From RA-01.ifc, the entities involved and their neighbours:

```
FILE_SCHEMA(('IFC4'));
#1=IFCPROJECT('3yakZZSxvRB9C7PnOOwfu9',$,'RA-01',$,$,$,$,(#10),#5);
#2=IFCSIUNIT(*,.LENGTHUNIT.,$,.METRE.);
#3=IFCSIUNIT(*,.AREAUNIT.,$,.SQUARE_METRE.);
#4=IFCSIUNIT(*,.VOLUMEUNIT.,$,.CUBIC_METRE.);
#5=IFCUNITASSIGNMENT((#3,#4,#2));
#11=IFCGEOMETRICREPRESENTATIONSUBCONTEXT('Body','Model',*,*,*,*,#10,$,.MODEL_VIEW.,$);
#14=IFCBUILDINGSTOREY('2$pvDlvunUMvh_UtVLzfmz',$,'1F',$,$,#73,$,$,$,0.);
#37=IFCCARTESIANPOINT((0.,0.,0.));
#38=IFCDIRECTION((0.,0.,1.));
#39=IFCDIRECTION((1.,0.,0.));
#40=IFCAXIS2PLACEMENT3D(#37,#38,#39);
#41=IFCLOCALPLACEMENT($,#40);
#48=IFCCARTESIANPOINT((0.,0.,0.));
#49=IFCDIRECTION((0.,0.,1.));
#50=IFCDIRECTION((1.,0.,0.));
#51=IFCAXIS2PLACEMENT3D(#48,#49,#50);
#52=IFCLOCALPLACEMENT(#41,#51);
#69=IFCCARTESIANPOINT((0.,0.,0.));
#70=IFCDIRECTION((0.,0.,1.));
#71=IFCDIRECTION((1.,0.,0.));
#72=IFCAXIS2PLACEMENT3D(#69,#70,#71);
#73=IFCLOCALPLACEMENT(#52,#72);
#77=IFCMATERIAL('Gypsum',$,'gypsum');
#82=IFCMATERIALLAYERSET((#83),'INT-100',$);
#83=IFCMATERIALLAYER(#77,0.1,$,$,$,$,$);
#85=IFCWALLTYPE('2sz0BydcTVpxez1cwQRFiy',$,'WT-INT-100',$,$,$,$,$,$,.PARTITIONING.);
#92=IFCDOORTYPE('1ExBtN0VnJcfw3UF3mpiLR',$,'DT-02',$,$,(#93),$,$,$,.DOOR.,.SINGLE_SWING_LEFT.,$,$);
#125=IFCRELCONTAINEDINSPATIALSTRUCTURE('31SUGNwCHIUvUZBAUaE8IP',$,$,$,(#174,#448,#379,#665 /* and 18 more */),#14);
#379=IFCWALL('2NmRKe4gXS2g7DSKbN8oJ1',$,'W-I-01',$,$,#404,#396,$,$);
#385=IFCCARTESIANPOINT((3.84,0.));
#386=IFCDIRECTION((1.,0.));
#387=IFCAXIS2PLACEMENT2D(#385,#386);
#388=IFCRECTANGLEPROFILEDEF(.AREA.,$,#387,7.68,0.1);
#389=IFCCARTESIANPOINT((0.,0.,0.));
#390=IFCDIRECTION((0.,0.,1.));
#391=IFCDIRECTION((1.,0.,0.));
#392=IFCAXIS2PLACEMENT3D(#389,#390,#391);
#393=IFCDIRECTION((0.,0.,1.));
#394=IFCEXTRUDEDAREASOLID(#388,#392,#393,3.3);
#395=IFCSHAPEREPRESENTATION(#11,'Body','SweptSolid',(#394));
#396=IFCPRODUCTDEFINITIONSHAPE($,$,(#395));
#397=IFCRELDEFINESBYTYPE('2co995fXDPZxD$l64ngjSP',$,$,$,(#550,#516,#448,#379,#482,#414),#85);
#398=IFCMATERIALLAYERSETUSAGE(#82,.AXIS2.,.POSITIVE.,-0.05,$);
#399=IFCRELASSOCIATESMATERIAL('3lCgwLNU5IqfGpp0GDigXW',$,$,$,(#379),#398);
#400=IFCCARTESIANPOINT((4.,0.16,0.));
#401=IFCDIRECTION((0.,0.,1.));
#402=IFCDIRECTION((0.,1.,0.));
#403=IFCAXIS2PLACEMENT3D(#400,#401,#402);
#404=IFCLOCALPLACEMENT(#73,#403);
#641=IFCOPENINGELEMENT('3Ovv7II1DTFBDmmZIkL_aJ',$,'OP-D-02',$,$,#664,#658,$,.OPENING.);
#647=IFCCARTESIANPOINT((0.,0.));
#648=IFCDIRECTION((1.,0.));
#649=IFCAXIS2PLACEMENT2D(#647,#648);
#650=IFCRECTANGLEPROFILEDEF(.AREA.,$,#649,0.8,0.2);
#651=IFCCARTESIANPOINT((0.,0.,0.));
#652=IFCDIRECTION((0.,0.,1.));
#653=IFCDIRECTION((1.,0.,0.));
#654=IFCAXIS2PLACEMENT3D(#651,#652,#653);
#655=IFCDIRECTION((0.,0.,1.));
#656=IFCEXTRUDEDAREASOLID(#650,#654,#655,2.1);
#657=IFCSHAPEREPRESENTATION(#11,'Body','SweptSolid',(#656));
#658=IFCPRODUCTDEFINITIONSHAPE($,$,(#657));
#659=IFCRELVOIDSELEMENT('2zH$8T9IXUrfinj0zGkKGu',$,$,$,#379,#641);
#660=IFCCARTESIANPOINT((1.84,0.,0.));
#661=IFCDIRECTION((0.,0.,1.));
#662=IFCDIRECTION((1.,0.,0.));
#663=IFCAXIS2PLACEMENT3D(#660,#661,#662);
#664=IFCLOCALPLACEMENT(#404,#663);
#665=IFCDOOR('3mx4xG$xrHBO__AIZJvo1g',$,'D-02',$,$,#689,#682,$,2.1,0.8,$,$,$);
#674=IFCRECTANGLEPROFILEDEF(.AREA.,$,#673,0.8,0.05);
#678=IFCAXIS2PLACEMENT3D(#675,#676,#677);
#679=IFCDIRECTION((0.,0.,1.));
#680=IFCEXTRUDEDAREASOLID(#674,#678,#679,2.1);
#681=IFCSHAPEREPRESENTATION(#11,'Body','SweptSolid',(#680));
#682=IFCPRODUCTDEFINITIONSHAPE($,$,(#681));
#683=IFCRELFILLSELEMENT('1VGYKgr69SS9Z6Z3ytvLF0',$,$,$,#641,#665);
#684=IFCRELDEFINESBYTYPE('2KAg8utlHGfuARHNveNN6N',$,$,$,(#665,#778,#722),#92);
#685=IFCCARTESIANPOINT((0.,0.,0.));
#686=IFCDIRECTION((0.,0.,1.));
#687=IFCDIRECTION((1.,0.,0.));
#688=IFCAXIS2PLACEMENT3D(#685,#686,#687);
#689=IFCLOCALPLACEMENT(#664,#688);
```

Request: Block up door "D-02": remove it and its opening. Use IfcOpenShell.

```python
import ifcopenshell
import ifcopenshell.api.feature
import ifcopenshell.api.root
import ifcopenshell.geom
import ifcopenshell.util.shape

model = ifcopenshell.open("RA-01.ifc")
settings = ifcopenshell.geom.settings()


def volume(element):
    """Net volume in cubic metres, openings subtracted."""
    shape = ifcopenshell.geom.create_shape(settings, element)
    return ifcopenshell.util.shape.get_volume(shape.geometry)


door = model.by_guid("3mx4xG$xrHBO__AIZJvo1g")
opening = door.FillsVoids[0].RelatingOpeningElement
wall = opening.VoidsElements[0].RelatingBuildingElement
before = volume(wall)

ifcopenshell.api.root.remove_product(model, product=door)
ifcopenshell.api.feature.remove_feature(model, feature=opening)

after = volume(wall)

print(f"wall volume {before:.3f} -> {after:.3f} m3")

model.write("RA-01_rev.ifc")
```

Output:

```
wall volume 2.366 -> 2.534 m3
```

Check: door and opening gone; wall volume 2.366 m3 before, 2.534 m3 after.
